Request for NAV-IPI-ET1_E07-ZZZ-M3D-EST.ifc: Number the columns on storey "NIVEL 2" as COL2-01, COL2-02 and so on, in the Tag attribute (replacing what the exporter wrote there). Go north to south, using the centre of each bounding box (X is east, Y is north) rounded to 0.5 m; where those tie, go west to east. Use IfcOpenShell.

First a look at what the model holds.

```python
import ifcopenshell
import ifcopenshell.util.element
import ifcopenshell.util.placement

model = ifcopenshell.open("NAV-IPI-ET1_E07-ZZZ-M3D-EST.ifc")
print(model.schema)
storey = next(s for s in model.by_type("IfcBuildingStorey") if s.Name == "NIVEL 2")
columns = [e for e in ifcopenshell.util.element.get_decomposition(storey) if e.is_a("IfcColumn")]
for e in sorted(columns, key=lambda e: e.id()):
    origin = ifcopenshell.util.placement.get_local_placement(e.ObjectPlacement)[:3, 3]
    print(e.id(), e.Tag, e.Name, origin.round(2) + 0.0, sep=" | ")
```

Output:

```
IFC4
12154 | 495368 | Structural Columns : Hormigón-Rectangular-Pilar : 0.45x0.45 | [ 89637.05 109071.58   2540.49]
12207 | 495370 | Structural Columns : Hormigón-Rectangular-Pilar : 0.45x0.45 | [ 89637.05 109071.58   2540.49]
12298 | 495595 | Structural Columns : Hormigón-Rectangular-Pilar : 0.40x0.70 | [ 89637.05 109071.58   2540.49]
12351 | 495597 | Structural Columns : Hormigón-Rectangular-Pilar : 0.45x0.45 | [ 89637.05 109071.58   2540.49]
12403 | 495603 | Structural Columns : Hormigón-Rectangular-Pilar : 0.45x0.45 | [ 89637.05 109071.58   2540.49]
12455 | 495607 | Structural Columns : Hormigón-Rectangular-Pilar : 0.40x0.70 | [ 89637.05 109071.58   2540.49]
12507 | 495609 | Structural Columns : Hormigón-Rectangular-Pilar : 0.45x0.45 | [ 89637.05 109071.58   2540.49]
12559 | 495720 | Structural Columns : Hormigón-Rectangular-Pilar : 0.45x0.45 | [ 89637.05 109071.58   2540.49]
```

```python
import ifcopenshell
import ifcopenshell.geom
import ifcopenshell.util.element
import ifcopenshell.util.shape

model = ifcopenshell.open("NAV-IPI-ET1_E07-ZZZ-M3D-EST.ifc")
settings = ifcopenshell.geom.settings()
settings.set("use-world-coords", True)


def centre(element):
    shape = ifcopenshell.geom.create_shape(settings, element)
    return ifcopenshell.util.shape.get_bbox_centroid(shape.geometry)


storey = next(s for s in model.by_type("IfcBuildingStorey") if s.Name == "NIVEL 2")
columns = [e for e in ifcopenshell.util.element.get_decomposition(storey) if e.is_a("IfcColumn")]

# Insertion points can sit at a corner or the storey origin, so sort by the geometry (in metres).
centres = {e: centre(e) for e in columns}
columns.sort(key=lambda e: (-round(centres[e][1] / 0.5), centres[e][0]))

for i, e in enumerate(columns, start=1):
    number = f"COL2-{i:02d}"
    e.Tag = number
    print(e.id(), number)

model.write("NAV-IPI-ET1_E07-ZZZ-M3D-EST_rev.ifc")
```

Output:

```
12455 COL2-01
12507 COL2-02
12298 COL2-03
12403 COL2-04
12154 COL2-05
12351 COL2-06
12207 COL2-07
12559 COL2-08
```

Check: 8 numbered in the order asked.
